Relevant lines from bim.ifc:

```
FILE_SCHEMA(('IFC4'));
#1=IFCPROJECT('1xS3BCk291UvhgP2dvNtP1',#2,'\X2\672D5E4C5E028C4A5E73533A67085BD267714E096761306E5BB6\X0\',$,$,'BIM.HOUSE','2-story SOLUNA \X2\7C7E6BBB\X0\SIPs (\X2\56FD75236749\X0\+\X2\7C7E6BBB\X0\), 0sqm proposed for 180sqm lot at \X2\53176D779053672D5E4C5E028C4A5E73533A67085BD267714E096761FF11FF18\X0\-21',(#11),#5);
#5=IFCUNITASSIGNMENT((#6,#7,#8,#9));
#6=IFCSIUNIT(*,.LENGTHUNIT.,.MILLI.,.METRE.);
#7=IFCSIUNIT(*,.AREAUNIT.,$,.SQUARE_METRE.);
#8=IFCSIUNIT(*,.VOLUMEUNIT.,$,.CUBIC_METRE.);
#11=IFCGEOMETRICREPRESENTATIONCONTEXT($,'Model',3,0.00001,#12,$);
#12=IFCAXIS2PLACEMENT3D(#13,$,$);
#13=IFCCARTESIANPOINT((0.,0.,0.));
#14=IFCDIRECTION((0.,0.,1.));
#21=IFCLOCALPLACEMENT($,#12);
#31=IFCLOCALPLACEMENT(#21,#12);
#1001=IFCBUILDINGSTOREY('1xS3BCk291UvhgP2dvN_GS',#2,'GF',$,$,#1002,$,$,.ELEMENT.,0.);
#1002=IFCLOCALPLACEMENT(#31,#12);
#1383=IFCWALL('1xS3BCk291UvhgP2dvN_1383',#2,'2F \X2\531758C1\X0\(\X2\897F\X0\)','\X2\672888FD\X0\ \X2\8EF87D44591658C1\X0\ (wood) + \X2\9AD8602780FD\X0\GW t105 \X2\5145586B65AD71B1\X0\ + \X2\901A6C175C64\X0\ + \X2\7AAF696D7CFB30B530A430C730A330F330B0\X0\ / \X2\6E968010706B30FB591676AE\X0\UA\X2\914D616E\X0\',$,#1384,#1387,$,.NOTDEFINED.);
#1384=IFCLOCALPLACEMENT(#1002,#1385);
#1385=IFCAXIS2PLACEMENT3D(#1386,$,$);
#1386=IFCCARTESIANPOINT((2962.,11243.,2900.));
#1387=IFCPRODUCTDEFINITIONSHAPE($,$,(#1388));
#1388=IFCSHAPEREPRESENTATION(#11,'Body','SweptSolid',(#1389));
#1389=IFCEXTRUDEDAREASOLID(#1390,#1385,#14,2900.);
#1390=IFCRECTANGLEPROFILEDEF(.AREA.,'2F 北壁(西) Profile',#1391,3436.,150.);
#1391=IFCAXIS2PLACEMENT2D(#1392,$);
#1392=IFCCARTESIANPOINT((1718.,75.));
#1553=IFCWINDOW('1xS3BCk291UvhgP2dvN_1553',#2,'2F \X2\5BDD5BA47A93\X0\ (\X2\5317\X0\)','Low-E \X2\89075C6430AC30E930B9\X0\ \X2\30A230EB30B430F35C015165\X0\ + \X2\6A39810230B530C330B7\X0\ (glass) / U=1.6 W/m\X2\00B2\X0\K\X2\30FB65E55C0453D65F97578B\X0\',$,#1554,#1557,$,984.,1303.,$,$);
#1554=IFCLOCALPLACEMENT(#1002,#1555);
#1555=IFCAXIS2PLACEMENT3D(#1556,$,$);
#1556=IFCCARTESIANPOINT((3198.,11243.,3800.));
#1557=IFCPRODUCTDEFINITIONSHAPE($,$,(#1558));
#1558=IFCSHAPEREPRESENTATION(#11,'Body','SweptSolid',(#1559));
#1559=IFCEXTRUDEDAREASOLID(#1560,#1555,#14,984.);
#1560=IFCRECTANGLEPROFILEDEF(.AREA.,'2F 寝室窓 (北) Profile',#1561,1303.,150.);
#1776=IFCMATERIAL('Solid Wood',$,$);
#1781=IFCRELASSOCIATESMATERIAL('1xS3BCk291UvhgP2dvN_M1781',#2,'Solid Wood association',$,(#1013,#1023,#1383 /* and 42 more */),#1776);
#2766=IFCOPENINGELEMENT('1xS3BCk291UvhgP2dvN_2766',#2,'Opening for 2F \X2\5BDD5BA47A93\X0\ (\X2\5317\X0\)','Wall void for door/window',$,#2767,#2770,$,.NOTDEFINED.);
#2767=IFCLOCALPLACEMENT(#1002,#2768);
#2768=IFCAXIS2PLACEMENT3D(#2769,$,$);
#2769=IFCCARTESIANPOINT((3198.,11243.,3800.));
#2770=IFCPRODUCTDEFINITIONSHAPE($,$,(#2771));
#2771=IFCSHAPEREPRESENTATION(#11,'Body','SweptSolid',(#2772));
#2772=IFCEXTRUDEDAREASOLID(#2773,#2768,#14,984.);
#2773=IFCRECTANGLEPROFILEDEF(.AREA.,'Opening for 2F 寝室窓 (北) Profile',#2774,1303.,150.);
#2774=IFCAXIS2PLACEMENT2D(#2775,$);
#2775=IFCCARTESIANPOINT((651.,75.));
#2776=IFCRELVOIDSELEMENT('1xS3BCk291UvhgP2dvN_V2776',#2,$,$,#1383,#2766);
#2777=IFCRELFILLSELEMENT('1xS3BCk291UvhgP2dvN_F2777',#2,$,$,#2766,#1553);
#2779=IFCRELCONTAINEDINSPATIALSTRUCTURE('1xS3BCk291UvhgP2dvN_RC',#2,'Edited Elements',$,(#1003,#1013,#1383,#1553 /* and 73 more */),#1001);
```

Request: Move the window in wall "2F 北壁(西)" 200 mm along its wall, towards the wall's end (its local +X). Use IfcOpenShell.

```python
import ifcopenshell
import ifcopenshell.api.geometry
import ifcopenshell.util.placement
import ifcopenshell.util.unit

model = ifcopenshell.open("bim.ifc")
unit_scale = ifcopenshell.util.unit.calculate_unit_scale(model)

window = model.by_id(1553)
opening = window.FillsVoids[0].RelatingOpeningElement
wall = opening.VoidsElements[0].RelatingBuildingElement

wall_matrix = ifcopenshell.util.placement.get_local_placement(wall.ObjectPlacement)
shift = wall_matrix[:3, 0] * 0.2 / unit_scale
before = ifcopenshell.util.placement.get_local_placement(window.ObjectPlacement)[:3, 3].copy()

# The window is not placed relative to its opening, so move both.
for product in (opening, window):
    matrix = ifcopenshell.util.placement.get_local_placement(product.ObjectPlacement)
    matrix[:3, 3] += shift
    ifcopenshell.api.geometry.edit_object_placement(model, product=product, matrix=matrix, is_si=False)

after = ifcopenshell.util.placement.get_local_placement(window.ObjectPlacement)[:3, 3]
print("window moved by", (after - before).round(3) + 0.0)

model.write("bim_rev.ifc")
```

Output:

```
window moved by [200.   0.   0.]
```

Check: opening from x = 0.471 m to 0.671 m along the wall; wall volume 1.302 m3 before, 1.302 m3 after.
